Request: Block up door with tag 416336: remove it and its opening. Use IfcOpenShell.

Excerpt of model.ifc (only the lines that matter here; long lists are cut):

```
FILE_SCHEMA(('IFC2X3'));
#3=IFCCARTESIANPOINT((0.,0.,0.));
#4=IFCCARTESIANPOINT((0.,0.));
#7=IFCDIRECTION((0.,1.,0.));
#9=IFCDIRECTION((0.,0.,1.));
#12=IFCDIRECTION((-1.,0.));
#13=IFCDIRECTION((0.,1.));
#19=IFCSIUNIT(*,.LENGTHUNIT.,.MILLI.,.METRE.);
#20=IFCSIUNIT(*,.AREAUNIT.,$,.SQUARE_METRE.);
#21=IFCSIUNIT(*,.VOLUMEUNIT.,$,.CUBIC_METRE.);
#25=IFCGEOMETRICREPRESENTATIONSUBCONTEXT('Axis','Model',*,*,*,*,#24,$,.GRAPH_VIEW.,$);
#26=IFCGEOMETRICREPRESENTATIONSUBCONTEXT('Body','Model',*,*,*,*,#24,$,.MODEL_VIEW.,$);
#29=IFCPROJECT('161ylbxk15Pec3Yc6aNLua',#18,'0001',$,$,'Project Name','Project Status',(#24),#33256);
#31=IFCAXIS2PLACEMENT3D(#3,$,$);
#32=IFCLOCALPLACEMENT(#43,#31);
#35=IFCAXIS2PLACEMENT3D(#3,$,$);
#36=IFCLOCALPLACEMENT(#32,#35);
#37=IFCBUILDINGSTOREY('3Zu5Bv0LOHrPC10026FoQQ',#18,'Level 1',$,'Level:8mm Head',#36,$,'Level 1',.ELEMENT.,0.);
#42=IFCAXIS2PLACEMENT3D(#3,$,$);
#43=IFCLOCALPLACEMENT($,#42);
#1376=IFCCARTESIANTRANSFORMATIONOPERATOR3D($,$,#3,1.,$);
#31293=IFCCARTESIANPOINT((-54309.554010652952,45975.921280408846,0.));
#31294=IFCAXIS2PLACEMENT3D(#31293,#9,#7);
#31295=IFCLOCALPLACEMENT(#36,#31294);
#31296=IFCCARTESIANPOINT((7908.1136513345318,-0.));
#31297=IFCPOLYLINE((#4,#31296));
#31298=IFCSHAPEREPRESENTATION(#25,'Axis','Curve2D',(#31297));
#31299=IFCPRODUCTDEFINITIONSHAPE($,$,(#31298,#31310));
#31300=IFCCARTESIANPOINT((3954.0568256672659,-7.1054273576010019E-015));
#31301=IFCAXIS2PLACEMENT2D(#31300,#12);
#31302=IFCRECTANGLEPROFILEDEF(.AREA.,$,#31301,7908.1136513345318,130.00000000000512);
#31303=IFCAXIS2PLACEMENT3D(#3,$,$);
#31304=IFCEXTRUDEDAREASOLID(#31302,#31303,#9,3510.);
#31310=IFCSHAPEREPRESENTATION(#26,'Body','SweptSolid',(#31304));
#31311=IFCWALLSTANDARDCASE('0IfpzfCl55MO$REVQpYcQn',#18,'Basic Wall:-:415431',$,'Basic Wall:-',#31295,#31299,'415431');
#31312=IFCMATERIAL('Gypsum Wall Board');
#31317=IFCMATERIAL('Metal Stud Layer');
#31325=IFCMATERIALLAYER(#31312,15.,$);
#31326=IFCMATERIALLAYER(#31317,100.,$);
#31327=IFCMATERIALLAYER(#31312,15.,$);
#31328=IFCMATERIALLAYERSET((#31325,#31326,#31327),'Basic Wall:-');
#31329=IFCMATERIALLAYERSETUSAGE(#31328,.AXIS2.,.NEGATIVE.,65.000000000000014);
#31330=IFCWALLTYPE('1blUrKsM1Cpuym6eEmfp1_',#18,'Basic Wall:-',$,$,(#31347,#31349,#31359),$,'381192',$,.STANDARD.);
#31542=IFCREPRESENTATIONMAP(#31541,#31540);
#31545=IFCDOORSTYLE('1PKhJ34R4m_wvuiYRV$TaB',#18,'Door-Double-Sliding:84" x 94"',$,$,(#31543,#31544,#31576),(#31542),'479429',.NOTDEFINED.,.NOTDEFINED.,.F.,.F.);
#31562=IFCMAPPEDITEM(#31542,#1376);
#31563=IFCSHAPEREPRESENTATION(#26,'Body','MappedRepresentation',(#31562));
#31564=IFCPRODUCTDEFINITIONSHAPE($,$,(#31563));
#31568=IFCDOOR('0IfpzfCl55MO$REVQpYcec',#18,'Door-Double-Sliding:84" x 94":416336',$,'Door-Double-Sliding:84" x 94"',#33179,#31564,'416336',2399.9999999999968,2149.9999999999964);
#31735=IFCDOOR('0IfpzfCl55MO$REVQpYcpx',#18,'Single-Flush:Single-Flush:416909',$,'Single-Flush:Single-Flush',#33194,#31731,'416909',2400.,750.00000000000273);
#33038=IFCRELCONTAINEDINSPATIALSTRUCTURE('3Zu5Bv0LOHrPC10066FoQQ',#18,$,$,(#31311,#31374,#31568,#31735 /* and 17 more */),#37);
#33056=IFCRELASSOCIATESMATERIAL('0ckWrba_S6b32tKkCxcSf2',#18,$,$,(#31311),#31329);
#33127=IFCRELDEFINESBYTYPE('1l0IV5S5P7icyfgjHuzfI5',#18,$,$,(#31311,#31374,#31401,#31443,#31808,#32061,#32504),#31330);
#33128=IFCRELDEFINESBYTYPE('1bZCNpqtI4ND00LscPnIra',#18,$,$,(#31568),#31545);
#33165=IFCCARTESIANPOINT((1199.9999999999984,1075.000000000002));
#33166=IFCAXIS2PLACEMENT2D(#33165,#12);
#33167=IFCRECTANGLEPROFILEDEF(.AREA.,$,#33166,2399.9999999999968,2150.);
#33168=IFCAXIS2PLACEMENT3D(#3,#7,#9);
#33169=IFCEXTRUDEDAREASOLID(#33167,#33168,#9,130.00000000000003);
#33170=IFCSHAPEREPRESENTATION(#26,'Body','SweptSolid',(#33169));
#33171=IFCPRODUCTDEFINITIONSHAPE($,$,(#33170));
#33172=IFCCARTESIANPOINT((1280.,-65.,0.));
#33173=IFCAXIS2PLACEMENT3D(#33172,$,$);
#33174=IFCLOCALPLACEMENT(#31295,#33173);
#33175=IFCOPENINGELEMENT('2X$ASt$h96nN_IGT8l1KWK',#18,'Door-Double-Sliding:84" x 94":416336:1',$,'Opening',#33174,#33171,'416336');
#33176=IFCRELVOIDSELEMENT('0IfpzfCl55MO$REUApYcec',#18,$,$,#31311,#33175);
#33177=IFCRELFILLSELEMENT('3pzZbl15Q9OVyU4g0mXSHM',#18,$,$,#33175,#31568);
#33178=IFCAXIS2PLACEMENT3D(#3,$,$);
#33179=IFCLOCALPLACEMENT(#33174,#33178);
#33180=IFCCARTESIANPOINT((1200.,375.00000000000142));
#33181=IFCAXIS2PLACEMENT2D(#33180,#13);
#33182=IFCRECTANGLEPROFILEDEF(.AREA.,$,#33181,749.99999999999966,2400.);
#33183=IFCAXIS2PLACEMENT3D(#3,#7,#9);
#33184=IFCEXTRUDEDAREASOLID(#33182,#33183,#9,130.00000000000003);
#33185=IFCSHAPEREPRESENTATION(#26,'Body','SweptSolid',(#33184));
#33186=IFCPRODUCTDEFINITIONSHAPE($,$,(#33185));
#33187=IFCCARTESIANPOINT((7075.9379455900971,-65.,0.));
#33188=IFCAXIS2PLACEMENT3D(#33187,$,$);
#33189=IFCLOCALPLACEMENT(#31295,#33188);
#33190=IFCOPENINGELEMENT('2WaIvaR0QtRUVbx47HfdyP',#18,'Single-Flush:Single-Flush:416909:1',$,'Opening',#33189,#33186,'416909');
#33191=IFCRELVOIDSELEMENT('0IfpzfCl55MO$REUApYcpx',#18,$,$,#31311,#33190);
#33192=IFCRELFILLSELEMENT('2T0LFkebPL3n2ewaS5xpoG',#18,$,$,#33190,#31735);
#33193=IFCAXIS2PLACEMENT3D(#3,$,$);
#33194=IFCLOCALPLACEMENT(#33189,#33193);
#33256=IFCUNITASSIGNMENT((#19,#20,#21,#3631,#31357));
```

```python
import ifcopenshell
import ifcopenshell.api.feature
import ifcopenshell.api.root
import ifcopenshell.geom
import ifcopenshell.util.shape

model = ifcopenshell.open("model.ifc")
settings = ifcopenshell.geom.settings()


def volume(element):
    """Net volume in cubic metres, openings subtracted."""
    shape = ifcopenshell.geom.create_shape(settings, element)
    return ifcopenshell.util.shape.get_volume(shape.geometry)


door = model.by_guid("0IfpzfCl55MO$REVQpYcec")
opening = door.FillsVoids[0].RelatingOpeningElement
wall = opening.VoidsElements[0].RelatingBuildingElement
before = volume(wall)

ifcopenshell.api.root.remove_product(model, product=door)
ifcopenshell.api.feature.remove_feature(model, feature=opening)

after = volume(wall)

print(f"wall volume {before:.3f} -> {after:.3f} m3")

model.write("model-out.ifc")
```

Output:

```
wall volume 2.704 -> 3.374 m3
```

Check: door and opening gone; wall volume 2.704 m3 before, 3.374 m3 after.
